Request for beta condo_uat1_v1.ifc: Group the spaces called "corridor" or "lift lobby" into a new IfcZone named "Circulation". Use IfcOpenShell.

First a look at what the model holds.

```python
import ifcopenshell

model = ifcopenshell.open("beta condo_uat1_v1.ifc")
print(model.schema)
seen = {}
for space in model.by_type("IfcSpace"):
    seen[space.LongName] = seen.get(space.LongName, 0) + 1
for name, count in sorted(seen.items(), key=str):
    print(count, "x", name)
print("zones:", [z.Name for z in model.by_type("IfcZone")][:20])
```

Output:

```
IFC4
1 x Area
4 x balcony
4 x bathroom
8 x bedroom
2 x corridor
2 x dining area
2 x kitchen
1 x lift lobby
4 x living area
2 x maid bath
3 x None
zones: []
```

```python
import ifcopenshell
import ifcopenshell.api.group
import ifcopenshell.api.root

model = ifcopenshell.open("beta condo_uat1_v1.ifc")

names = {"corridor", "lift lobby"}
spaces = [s for s in model.by_type("IfcSpace") if s.LongName in names]

zone = ifcopenshell.api.root.create_entity(model, ifc_class="IfcZone", name="Circulation")
ifcopenshell.api.group.assign_group(model, products=spaces, group=zone)
print(len(spaces), "spaces in", zone.Name)

model.write("beta condo_uat1_v1_rev.ifc")
```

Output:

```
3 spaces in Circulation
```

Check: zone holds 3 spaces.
